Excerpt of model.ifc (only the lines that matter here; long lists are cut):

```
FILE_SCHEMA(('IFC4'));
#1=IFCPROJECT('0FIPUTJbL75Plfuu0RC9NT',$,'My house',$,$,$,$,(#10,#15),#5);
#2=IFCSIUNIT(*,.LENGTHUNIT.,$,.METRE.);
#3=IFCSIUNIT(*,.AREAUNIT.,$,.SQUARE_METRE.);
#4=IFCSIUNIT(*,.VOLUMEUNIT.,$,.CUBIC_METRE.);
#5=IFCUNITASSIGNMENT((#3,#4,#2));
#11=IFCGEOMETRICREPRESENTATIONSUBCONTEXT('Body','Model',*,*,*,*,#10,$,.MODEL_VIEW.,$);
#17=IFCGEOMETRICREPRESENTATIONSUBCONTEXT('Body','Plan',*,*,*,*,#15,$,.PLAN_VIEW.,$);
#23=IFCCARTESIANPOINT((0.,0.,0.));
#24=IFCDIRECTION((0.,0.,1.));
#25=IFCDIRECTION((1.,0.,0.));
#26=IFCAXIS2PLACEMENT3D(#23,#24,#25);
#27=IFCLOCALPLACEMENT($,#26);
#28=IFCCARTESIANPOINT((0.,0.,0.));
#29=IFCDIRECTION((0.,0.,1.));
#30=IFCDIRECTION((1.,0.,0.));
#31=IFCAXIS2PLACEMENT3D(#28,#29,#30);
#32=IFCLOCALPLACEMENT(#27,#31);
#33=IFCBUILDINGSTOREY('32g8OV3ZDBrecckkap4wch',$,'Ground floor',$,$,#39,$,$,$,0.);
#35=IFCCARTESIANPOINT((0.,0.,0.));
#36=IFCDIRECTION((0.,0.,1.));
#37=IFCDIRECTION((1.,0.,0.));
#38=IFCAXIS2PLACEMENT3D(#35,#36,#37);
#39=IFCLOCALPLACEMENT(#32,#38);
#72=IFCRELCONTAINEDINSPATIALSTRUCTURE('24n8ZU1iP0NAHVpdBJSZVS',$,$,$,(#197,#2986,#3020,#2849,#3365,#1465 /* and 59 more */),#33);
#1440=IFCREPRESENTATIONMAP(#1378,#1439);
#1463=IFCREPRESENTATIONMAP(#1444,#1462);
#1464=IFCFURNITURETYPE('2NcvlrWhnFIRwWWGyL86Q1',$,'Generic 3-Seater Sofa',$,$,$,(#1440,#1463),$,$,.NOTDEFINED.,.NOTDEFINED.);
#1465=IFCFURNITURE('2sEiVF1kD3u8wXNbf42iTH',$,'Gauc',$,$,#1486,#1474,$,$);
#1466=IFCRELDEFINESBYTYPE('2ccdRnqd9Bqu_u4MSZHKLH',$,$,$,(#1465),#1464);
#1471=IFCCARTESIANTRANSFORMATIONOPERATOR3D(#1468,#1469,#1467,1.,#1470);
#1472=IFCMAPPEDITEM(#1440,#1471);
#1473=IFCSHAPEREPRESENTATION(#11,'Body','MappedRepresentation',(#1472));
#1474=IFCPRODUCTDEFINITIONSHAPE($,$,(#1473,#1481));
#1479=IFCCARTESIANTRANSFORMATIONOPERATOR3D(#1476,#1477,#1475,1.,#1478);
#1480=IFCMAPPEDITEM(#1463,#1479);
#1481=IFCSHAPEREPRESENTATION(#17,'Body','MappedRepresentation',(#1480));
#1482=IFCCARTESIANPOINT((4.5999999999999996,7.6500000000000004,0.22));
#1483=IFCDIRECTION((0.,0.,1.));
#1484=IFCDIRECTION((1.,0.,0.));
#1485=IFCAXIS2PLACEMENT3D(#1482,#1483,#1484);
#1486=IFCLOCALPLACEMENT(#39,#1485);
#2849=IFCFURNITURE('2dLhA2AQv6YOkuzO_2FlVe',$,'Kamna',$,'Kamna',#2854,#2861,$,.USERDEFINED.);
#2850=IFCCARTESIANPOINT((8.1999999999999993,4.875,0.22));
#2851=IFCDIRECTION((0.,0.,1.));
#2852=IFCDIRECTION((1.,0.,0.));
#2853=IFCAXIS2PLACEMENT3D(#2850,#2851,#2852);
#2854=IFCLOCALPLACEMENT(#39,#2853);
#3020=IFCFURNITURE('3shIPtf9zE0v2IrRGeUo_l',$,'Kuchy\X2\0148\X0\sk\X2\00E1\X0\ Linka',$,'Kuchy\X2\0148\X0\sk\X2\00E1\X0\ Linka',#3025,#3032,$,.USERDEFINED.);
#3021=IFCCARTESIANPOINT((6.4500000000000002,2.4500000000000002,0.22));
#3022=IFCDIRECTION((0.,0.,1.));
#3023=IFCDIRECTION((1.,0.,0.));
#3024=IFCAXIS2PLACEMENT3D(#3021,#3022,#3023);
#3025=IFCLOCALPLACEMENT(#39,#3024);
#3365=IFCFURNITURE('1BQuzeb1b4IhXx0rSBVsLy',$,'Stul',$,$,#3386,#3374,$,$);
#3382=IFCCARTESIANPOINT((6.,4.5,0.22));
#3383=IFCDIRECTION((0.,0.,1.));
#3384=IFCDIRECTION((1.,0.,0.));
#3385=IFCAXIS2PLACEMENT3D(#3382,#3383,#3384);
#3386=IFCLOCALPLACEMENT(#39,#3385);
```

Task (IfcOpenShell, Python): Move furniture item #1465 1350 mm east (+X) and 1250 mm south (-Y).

```python
import ifcopenshell
import ifcopenshell.api.geometry
import ifcopenshell.util.placement

model = ifcopenshell.open("model.ifc")

item = model.by_guid("2sEiVF1kD3u8wXNbf42iTH")
matrix = ifcopenshell.util.placement.get_local_placement(item.ObjectPlacement)
matrix[0, 3] += 1.35
matrix[1, 3] -= 1.25
ifcopenshell.api.geometry.edit_object_placement(model, product=item, matrix=matrix, is_si=False)

print(ifcopenshell.util.placement.get_local_placement(item.ObjectPlacement).round(3) + 0.0)

model.write("model_v2.ifc")
```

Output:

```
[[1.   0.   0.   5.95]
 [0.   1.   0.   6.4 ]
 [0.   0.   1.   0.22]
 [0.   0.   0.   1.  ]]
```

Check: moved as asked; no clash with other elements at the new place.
